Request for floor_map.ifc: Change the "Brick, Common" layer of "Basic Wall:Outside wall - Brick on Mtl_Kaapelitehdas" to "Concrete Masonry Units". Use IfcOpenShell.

First a look at what the model holds.

```python
import ifcopenshell
import ifcopenshell.util.element

model = ifcopenshell.open("floor_map.ifc")
print(model.schema)
for layer_set in model.by_type("IfcMaterialLayerSet"):
    if layer_set.LayerSetName == "Basic Wall:Outside wall - Brick on Mtl_Kaapelitehdas":
        for layer in layer_set.MaterialLayers:
            print(layer.id(), layer.Material and layer.Material.Name, layer.LayerThickness, sep=" | ")
        print(len(ifcopenshell.util.element.get_elements_by_material(model, layer_set)), "elements and types use it")
print(sorted(m.Name for m in model.by_type("IfcMaterial") if m.Name)[:60])
```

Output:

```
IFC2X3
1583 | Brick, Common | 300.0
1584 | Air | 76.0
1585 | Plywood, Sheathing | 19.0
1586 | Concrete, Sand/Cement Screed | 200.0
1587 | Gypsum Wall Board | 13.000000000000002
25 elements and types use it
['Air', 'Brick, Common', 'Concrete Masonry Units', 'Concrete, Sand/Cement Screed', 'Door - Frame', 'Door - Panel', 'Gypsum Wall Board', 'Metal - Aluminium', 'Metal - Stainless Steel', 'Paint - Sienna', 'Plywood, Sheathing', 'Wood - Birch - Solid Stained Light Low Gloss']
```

```python
import ifcopenshell
import ifcopenshell.api.material

model = ifcopenshell.open("floor_map.ifc")

layer_set = next(s for s in model.by_type("IfcMaterialLayerSet") if s.LayerSetName == "Basic Wall:Outside wall - Brick on Mtl_Kaapelitehdas")
layer = next(l for l in layer_set.MaterialLayers if l.Material and l.Material.Name == "Brick, Common")
material = next(m for m in model.by_type("IfcMaterial") if m.Name == "Concrete Masonry Units")

# Point this one layer at the other material; renaming the old one would change it everywhere.
ifcopenshell.api.material.edit_layer(model, layer=layer, attributes={}, material=material)

print([l.Material.Name if l.Material else None for l in layer_set.MaterialLayers])

model.write("floor_map_v2.ifc")
```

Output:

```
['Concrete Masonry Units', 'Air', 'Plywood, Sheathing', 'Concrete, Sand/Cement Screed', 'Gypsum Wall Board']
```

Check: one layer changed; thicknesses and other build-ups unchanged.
